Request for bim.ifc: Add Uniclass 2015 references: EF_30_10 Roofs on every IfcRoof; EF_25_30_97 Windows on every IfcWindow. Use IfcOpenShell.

First a look at what the model holds.

```python
import ifcopenshell

model = ifcopenshell.open("bim.ifc")
print(model.schema)
print("classifications:", [c.Name for c in model.by_type("IfcClassification")])
for ifc_class in ("IfcDoor", "IfcRoof", "IfcStair", "IfcWall", "IfcWindow"):
    print(ifc_class, len(model.by_type(ifc_class)))
```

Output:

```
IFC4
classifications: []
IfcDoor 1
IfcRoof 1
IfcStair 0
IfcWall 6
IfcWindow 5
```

```python
import ifcopenshell
import ifcopenshell.api.classification

model = ifcopenshell.open("bim.ifc")

system = ifcopenshell.api.classification.add_classification(model, classification="Uniclass 2015")

codes = {
    "IfcRoof": ("EF_30_10", "Roofs"),
    "IfcWindow": ("EF_25_30_97", "Windows"),
}
for ifc_class, (code, name) in codes.items():
    products = model.by_type(ifc_class)
    ifcopenshell.api.classification.add_reference(
        model, products=products, classification=system, identification=code, name=name
    )
    print(code, len(products))

model.write("bim_v2.ifc")
```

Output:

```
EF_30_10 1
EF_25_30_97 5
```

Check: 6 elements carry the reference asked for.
